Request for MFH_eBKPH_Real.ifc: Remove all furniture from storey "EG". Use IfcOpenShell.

First a look at what the model holds.

```python
import ifcopenshell
import ifcopenshell.util.element

model = ifcopenshell.open("MFH_eBKPH_Real.ifc")
print(model.schema)
storey = next(s for s in model.by_type("IfcBuildingStorey") if s.Name == "EG")
furniture = [e for e in ifcopenshell.util.element.get_decomposition(storey) if e.is_a("IfcFurnishingElement")]
seen = {}
for e in furniture:
    element_type = ifcopenshell.util.element.get_type(e)
    name = element_type.Name if element_type not in (None, e) else None
    seen[name] = seen.get(name, 0) + 1
for name, count in sorted(seen.items(), key=str):
    print(count, "x", name)
```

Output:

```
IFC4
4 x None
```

```python
import ifcopenshell
import ifcopenshell.api.root
import ifcopenshell.util.element

model = ifcopenshell.open("MFH_eBKPH_Real.ifc")

storey = next(s for s in model.by_type("IfcBuildingStorey") if s.Name == "EG")
furniture = [e for e in ifcopenshell.util.element.get_decomposition(storey) if e.is_a("IfcFurnishingElement")]

for e in furniture:
    ifcopenshell.api.root.remove_product(model, product=e)
print(len(furniture), "removed")

model.write("MFH_eBKPH_Real_edited.ifc")
```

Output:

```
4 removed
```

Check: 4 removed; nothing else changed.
